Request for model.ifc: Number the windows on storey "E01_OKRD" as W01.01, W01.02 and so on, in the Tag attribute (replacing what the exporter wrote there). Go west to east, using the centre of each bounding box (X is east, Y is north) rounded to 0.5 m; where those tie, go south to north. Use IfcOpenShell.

First a look at what the model holds.

```python
import ifcopenshell
import ifcopenshell.util.element
import ifcopenshell.util.placement

model = ifcopenshell.open("model.ifc")
print(model.schema)
storey = next(s for s in model.by_type("IfcBuildingStorey") if s.Name == "E01_OKRD")
windows = [e for e in ifcopenshell.util.element.get_decomposition(storey) if e.is_a("IfcWindow")]
for e in sorted(windows, key=lambda e: e.id()):
    origin = ifcopenshell.util.placement.get_local_placement(e.ObjectPlacement)[:3, 3]
    print(e.id(), e.Tag, e.Name, origin.round(2) + 0.0, sep=" | ")
```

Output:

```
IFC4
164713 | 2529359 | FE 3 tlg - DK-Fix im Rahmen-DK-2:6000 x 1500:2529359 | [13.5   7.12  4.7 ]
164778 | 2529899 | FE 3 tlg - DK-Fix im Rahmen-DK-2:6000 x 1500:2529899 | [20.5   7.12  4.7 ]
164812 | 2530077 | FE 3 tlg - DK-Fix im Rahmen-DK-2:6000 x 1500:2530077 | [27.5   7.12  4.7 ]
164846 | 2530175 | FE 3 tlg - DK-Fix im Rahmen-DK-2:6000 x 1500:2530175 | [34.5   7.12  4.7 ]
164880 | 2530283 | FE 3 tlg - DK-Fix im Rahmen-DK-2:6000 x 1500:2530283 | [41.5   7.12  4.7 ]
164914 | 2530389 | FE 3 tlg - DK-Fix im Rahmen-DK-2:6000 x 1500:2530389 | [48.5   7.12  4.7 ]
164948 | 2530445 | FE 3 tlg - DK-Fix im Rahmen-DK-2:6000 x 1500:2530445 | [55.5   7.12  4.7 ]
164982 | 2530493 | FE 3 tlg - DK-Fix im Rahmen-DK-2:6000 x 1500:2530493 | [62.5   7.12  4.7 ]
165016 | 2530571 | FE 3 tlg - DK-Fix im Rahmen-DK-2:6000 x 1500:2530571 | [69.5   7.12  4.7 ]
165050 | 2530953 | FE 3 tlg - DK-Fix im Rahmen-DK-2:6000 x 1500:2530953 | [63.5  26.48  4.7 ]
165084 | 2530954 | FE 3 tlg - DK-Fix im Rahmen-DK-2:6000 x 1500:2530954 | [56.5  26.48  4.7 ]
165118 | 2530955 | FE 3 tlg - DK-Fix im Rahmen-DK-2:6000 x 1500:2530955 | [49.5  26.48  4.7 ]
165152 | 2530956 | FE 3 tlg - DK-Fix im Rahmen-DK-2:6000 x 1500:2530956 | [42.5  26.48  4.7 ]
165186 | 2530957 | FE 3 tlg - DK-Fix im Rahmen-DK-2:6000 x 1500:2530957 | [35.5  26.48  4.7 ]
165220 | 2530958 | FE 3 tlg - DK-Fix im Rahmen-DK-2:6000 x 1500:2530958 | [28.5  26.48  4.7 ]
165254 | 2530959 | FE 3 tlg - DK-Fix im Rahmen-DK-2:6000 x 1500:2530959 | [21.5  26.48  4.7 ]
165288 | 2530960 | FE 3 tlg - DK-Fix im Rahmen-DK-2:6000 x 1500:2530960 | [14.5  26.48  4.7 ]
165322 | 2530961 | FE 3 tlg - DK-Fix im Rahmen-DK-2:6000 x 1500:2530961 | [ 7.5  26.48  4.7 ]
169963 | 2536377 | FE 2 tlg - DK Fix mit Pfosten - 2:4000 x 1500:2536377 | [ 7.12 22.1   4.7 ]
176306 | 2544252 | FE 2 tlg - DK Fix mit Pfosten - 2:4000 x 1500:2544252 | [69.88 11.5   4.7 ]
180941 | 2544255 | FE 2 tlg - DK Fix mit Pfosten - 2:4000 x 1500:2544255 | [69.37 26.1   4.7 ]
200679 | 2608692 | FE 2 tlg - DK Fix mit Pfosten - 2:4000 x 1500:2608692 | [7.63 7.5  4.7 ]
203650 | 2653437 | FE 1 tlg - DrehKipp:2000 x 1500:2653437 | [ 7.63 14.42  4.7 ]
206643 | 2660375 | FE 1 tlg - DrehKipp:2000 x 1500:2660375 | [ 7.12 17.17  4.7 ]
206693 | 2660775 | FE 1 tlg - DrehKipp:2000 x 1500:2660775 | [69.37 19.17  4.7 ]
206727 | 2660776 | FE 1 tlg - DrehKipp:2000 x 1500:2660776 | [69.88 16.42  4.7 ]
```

```python
import ifcopenshell
import ifcopenshell.geom
import ifcopenshell.util.element
import ifcopenshell.util.shape

model = ifcopenshell.open("model.ifc")
settings = ifcopenshell.geom.settings()
settings.set("use-world-coords", True)


def centre(element):
    shape = ifcopenshell.geom.create_shape(settings, element)
    return ifcopenshell.util.shape.get_bbox_centroid(shape.geometry)


storey = next(s for s in model.by_type("IfcBuildingStorey") if s.Name == "E01_OKRD")
windows = [e for e in ifcopenshell.util.element.get_decomposition(storey) if e.is_a("IfcWindow")]

# Insertion points can sit at a corner or the storey origin, so sort by the geometry (in metres).
centres = {e: centre(e) for e in windows}
windows.sort(key=lambda e: (round(centres[e][0] / 0.5), centres[e][1]))

for i, e in enumerate(windows, start=1):
    number = f"W01.{i:02d}"
    e.Tag = number
    print(e.id(), number)

model.write("model_edited.ifc")
```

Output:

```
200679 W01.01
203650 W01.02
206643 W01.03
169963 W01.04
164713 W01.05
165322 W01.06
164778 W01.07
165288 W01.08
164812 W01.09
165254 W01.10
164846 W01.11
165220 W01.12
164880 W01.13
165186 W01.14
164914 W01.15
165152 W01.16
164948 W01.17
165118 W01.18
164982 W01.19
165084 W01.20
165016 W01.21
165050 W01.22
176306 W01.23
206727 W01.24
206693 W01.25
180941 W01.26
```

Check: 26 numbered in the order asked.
